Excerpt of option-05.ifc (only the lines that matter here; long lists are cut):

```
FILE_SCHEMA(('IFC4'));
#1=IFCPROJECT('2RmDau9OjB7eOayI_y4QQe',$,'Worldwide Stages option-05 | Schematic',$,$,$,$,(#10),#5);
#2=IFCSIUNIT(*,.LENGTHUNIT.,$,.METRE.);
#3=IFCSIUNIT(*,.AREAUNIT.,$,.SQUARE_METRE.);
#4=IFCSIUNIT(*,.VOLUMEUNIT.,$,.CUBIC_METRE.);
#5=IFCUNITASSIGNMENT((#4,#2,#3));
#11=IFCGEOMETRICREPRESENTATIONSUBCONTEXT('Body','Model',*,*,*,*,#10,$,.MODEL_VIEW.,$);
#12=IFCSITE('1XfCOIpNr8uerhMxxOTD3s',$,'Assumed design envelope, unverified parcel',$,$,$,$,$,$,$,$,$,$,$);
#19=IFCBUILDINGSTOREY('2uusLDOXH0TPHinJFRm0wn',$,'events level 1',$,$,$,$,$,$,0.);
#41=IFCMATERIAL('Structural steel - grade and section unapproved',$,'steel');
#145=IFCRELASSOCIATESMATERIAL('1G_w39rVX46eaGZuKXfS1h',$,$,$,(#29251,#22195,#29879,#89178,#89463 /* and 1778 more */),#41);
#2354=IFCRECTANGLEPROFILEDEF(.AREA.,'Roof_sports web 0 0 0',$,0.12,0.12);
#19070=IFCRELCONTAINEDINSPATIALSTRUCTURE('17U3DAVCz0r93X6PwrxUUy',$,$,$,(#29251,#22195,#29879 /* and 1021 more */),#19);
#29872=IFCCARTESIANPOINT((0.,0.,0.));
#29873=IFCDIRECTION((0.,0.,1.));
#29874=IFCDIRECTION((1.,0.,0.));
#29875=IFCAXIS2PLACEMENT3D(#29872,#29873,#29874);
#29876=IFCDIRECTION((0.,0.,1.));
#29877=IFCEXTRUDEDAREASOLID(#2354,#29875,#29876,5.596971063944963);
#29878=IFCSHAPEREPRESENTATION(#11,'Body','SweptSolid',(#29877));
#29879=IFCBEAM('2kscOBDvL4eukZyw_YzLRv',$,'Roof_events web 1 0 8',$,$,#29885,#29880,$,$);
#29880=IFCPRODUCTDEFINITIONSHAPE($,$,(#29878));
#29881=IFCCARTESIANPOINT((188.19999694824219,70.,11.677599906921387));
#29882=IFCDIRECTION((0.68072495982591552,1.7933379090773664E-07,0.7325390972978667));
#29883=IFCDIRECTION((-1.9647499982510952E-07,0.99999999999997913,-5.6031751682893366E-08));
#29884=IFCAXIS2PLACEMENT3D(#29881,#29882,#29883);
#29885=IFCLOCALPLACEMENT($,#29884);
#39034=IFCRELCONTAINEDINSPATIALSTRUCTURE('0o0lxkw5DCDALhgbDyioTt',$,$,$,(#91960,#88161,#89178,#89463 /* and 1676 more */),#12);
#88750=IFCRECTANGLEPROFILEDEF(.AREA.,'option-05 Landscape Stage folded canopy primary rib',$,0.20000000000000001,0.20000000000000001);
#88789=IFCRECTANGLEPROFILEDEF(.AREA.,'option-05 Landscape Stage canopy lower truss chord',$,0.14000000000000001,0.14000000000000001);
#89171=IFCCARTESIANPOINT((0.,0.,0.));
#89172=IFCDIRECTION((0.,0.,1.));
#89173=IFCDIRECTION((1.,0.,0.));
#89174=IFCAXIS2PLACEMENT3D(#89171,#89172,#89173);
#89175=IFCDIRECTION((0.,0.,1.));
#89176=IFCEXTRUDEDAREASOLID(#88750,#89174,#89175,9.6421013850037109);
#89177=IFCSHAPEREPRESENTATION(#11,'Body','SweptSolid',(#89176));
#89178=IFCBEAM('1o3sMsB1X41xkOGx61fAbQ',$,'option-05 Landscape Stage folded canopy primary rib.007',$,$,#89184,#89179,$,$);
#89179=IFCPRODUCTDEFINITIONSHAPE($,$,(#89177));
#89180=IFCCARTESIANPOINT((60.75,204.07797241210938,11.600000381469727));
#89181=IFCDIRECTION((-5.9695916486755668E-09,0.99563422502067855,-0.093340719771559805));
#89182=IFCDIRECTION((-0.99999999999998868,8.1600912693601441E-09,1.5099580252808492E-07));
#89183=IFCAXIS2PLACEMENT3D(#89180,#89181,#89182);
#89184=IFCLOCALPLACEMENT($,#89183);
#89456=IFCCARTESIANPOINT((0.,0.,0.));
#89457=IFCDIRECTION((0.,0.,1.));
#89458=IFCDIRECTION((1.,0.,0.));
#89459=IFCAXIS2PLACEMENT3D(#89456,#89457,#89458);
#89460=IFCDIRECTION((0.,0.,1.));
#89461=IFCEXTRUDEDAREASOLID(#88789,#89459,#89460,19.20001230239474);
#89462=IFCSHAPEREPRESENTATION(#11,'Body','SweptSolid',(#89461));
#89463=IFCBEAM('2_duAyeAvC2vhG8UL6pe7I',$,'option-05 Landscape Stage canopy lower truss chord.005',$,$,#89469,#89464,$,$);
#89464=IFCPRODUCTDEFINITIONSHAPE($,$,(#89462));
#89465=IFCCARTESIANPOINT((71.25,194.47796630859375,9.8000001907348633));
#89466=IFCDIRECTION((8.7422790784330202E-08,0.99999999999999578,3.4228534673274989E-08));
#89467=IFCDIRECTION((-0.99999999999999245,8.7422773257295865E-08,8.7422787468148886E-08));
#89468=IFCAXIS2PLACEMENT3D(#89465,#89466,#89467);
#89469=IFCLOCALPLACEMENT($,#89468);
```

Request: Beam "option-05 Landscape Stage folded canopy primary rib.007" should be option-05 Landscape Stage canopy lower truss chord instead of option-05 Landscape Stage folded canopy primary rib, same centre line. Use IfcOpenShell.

```python
import ifcopenshell
import ifcopenshell.util.element
import ifcopenshell.util.representation

model = ifcopenshell.open("option-05.ifc")

member = model.by_guid("1o3sMsB1X41xkOGx61fAbQ")
source = next(p for p in model.by_type("IfcRectangleProfileDef") if p.ProfileName == "option-05 Landscape Stage canopy lower truss chord")

body = ifcopenshell.util.representation.get_representation(member, "Model", "Body")
solid = body.Items[0]
old_profile = solid.SweptArea

# Copy the section's sizes but keep this member's own profile position.
profile = ifcopenshell.util.element.copy(model, source)
profile.Position = old_profile.Position
solid.SweptArea = profile
if not model.get_total_inverses(old_profile):
    ifcopenshell.util.element.remove_deep2(model, old_profile)
member.Name = member.Name.replace("option-05 Landscape Stage folded canopy primary rib", "option-05 Landscape Stage canopy lower truss chord")

print(solid.SweptArea)

model.write("option-05_rev.ifc")
```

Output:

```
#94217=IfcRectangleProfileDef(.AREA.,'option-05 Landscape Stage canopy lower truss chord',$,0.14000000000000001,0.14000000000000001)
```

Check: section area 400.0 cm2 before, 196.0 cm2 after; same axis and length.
